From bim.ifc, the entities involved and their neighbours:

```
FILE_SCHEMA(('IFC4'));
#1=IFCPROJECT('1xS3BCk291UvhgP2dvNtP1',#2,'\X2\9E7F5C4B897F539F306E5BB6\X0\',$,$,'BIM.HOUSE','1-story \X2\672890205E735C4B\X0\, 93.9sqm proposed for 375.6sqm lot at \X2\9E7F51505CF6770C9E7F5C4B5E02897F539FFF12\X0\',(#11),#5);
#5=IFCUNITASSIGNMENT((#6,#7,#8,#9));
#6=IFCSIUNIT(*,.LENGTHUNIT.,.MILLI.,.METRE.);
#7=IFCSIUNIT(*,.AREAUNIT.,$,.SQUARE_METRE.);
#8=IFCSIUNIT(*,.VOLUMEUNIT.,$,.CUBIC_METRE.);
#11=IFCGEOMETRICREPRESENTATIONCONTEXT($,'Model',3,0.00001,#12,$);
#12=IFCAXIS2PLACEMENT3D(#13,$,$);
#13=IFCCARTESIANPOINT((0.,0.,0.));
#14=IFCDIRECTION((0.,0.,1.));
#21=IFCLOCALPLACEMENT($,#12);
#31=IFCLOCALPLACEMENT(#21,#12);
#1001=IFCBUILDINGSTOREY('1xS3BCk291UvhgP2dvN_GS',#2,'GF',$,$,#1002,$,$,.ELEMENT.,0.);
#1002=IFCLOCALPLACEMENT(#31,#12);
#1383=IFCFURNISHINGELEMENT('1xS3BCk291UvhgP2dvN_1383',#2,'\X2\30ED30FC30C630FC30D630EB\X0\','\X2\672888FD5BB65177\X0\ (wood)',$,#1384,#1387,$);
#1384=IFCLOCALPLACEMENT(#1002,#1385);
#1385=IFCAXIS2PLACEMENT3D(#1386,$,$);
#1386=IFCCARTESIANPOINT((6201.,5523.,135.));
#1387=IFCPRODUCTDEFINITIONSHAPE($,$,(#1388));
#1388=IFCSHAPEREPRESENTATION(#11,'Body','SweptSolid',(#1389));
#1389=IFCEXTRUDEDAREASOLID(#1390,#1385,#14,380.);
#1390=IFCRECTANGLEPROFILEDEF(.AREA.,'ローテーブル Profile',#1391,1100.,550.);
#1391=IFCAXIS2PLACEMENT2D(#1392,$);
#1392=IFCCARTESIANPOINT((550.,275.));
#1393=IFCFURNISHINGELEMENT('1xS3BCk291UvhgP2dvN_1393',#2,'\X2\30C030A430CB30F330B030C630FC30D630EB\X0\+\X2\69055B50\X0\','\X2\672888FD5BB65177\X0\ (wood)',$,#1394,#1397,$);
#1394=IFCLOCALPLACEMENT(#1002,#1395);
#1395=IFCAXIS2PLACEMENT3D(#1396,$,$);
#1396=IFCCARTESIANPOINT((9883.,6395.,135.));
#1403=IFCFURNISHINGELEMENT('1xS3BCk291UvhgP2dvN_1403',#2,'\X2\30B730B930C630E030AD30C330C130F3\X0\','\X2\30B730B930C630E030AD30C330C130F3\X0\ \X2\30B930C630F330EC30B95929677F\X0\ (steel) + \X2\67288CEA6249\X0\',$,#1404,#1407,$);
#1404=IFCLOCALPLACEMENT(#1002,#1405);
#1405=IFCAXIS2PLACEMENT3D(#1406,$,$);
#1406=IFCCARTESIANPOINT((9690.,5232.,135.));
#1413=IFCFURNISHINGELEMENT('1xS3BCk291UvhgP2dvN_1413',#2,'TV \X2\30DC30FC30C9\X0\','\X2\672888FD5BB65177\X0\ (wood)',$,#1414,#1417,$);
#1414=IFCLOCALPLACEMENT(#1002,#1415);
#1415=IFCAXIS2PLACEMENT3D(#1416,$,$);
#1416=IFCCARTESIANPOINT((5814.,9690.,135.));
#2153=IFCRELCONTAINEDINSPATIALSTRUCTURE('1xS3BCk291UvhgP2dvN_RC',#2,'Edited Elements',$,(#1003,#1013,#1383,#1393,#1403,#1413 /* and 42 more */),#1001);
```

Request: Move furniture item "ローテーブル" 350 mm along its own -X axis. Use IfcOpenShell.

```python
import ifcopenshell
import ifcopenshell.api.geometry
import ifcopenshell.util.placement
import ifcopenshell.util.unit

model = ifcopenshell.open("bim.ifc")
unit_scale = ifcopenshell.util.unit.calculate_unit_scale(model)

item = model.by_id(1383)
matrix = ifcopenshell.util.placement.get_local_placement(item.ObjectPlacement)
matrix[:3, 3] -= matrix[:3, 0] * 0.35 / unit_scale
ifcopenshell.api.geometry.edit_object_placement(model, product=item, matrix=matrix, is_si=False)

print(ifcopenshell.util.placement.get_local_placement(item.ObjectPlacement).round(3) + 0.0)

model.write("bim_edited.ifc")
```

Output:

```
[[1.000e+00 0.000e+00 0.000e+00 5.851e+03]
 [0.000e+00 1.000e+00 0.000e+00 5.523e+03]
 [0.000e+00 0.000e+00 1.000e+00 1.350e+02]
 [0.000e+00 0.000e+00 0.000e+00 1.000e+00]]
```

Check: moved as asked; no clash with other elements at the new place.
